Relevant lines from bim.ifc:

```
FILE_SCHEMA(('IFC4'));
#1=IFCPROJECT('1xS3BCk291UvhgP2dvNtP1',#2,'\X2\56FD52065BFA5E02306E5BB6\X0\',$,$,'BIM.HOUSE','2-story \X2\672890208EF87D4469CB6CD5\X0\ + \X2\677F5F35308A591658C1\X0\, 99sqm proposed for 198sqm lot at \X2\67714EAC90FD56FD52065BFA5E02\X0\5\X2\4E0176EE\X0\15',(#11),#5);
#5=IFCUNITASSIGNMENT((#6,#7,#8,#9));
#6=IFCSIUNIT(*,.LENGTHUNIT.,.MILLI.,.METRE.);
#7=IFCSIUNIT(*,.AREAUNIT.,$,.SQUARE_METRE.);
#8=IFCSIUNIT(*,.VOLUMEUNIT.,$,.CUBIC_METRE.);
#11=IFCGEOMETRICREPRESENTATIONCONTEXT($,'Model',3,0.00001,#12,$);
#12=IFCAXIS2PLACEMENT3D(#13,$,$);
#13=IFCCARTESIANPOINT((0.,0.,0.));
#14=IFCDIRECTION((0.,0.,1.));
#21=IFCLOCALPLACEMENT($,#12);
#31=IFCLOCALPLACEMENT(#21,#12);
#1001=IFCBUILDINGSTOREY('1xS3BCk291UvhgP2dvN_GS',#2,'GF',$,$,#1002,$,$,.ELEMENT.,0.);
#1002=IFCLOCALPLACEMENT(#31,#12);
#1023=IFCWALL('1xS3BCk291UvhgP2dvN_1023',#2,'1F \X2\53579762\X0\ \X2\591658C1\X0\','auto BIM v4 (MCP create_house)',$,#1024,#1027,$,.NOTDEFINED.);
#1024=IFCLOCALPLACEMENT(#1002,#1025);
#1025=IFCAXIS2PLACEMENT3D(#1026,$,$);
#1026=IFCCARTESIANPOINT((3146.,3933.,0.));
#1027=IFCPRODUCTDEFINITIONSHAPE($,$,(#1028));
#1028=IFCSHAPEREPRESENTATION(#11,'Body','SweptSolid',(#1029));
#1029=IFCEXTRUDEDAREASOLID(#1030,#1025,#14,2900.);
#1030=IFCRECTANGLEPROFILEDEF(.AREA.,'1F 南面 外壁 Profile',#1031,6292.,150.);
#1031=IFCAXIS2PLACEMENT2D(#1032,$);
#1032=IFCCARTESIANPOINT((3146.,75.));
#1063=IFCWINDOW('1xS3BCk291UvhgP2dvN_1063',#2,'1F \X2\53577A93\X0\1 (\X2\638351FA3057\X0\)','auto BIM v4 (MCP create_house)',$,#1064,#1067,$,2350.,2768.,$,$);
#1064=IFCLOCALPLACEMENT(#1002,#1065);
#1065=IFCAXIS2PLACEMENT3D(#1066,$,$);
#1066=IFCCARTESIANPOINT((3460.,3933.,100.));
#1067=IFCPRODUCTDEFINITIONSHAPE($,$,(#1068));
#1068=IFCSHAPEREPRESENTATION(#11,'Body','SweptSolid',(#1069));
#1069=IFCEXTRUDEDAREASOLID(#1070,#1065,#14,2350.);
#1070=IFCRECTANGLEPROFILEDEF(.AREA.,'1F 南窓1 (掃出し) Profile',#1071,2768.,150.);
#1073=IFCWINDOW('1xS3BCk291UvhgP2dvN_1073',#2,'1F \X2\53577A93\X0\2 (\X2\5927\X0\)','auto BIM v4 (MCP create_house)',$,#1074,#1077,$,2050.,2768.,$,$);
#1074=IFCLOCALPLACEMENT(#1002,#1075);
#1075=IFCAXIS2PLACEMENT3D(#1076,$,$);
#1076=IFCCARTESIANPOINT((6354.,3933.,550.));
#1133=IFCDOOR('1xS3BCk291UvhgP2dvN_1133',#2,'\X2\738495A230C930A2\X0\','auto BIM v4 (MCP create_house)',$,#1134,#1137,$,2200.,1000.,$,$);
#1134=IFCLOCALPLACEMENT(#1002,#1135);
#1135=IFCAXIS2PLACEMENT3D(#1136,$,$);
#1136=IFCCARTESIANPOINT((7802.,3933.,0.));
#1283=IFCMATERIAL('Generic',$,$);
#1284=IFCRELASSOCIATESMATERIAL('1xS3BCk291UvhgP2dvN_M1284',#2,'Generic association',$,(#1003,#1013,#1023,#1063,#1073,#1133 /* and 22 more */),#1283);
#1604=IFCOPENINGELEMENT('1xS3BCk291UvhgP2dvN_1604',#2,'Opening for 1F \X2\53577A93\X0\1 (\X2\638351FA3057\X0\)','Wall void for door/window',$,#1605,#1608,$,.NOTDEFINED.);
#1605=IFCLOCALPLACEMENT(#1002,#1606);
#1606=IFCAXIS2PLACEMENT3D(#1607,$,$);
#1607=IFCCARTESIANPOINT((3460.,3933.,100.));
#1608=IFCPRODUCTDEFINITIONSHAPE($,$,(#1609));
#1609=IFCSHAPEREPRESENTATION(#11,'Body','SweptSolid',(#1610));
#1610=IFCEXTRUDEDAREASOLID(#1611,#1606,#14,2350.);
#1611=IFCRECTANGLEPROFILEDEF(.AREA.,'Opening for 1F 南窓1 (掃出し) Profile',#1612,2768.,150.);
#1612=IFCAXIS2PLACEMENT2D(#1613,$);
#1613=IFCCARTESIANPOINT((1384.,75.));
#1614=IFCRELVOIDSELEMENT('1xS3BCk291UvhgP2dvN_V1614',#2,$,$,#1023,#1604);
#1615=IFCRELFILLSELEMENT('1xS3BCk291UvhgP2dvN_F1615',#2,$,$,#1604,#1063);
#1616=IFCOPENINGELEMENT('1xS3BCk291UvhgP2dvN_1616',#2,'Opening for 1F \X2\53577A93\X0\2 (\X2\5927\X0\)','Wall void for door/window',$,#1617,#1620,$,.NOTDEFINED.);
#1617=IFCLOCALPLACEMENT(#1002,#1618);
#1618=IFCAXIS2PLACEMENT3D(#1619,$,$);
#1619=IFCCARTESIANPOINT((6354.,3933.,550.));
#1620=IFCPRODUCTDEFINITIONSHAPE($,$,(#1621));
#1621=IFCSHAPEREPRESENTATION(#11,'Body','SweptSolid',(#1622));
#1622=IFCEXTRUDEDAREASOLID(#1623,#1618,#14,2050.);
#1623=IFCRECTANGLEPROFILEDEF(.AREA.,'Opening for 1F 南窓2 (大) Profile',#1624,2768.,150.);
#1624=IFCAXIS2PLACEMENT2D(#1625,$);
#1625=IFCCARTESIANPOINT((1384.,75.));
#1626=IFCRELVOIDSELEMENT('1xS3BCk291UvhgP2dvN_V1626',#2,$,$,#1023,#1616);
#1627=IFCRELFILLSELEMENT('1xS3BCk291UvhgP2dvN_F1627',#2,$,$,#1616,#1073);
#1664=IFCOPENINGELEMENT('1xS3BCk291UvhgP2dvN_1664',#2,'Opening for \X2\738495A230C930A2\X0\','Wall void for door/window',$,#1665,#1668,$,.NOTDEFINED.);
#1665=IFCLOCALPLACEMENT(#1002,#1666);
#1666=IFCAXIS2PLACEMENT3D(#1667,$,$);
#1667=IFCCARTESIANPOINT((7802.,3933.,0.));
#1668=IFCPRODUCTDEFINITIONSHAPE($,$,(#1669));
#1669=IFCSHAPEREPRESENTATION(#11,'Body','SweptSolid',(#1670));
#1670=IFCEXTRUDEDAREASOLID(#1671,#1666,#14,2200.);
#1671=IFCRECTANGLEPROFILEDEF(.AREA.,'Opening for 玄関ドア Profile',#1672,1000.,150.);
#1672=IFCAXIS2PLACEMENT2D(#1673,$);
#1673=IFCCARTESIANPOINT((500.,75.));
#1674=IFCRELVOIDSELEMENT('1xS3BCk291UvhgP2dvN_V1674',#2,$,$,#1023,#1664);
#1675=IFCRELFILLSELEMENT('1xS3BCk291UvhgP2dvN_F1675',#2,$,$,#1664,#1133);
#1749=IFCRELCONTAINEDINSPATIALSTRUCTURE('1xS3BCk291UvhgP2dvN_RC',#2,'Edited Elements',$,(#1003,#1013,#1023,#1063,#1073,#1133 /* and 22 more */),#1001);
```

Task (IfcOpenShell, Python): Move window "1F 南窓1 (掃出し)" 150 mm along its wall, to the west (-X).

```python
import ifcopenshell
import ifcopenshell.api.geometry
import ifcopenshell.util.placement
import ifcopenshell.util.unit

model = ifcopenshell.open("bim.ifc")
unit_scale = ifcopenshell.util.unit.calculate_unit_scale(model)

window = model.by_guid("1xS3BCk291UvhgP2dvN_1063")
opening = window.FillsVoids[0].RelatingOpeningElement
wall = opening.VoidsElements[0].RelatingBuildingElement

wall_matrix = ifcopenshell.util.placement.get_local_placement(wall.ObjectPlacement)
shift = wall_matrix[:3, 0] * -0.15 / unit_scale
before = ifcopenshell.util.placement.get_local_placement(window.ObjectPlacement)[:3, 3].copy()

# The window is not placed relative to its opening, so move both.
for product in (opening, window):
    matrix = ifcopenshell.util.placement.get_local_placement(product.ObjectPlacement)
    matrix[:3, 3] += shift
    ifcopenshell.api.geometry.edit_object_placement(model, product=product, matrix=matrix, is_si=False)

after = ifcopenshell.util.placement.get_local_placement(window.ObjectPlacement)[:3, 3]
print("window moved by", (after - before).round(3) + 0.0)

model.write("bim_updated.ifc")
```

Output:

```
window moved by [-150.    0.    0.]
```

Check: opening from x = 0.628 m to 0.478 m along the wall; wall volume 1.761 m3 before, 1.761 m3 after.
